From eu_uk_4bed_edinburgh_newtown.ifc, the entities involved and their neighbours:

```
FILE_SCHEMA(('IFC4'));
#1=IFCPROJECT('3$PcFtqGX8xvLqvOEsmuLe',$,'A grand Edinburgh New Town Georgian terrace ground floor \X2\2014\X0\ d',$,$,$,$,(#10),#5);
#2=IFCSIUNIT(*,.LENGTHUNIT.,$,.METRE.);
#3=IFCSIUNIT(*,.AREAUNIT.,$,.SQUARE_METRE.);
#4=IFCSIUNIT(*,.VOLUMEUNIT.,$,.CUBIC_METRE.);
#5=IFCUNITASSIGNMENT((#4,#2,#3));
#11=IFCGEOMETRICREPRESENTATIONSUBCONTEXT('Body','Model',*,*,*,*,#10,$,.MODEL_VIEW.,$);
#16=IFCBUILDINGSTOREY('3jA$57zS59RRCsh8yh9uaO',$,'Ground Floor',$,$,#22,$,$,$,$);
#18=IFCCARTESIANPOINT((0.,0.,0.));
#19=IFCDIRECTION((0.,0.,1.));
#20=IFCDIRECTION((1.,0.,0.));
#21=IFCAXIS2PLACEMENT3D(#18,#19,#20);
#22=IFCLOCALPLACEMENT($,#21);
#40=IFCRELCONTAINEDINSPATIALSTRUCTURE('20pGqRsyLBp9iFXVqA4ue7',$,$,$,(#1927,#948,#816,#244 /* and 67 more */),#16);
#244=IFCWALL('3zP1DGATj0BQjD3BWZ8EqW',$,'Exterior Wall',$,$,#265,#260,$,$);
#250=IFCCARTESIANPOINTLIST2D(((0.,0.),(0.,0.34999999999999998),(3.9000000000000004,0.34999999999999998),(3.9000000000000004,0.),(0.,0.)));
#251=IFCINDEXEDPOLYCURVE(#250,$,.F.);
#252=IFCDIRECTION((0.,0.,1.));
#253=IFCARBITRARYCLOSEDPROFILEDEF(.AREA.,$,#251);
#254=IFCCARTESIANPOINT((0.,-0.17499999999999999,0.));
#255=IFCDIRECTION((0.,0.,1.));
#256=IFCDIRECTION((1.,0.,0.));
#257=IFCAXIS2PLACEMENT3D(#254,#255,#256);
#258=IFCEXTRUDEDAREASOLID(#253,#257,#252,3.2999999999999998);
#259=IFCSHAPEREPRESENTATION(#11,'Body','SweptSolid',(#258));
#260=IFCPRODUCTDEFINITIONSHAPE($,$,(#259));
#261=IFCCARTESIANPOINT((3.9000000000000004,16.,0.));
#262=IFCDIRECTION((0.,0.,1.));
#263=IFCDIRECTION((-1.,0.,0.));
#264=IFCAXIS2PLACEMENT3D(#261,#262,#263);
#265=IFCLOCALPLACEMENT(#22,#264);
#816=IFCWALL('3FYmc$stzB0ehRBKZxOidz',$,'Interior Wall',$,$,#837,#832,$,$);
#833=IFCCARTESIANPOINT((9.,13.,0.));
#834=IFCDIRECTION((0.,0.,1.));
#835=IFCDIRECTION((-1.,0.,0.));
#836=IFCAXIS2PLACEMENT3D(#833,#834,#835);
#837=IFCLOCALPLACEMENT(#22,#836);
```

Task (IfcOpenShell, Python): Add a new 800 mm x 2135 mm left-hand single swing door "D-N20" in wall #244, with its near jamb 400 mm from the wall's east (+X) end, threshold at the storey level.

```python
import numpy as np
import ifcopenshell
import ifcopenshell.api.feature
import ifcopenshell.api.geometry
import ifcopenshell.api.root
import ifcopenshell.api.spatial
import ifcopenshell.geom
import ifcopenshell.util.element
import ifcopenshell.util.placement
import ifcopenshell.util.representation
import ifcopenshell.util.shape
import ifcopenshell.util.unit

model = ifcopenshell.open("eu_uk_4bed_edinburgh_newtown.ifc")
unit_scale = ifcopenshell.util.unit.calculate_unit_scale(model)
settings = ifcopenshell.geom.settings()


def volume(element):
    """Net volume in cubic metres, openings subtracted."""
    shape = ifcopenshell.geom.create_shape(settings, element)
    return ifcopenshell.util.shape.get_volume(shape.geometry)


wall = model.by_guid("3zP1DGATj0BQjD3BWZ8EqW")
storey = ifcopenshell.util.element.get_container(wall, ifc_class="IfcBuildingStorey")
context = ifcopenshell.util.representation.get_context(model, "Model", "Body", "MODEL_VIEW")
before = volume(wall)

width, height, from_end, sill = 0.8, 2.135, 0.4, 0.0  # metres

# The wall runs along its own X axis, and the end named is its -X end.
wall_shape = ifcopenshell.geom.create_shape(settings, wall)
x, y, z = ifcopenshell.util.shape.get_vertices(wall_shape.geometry).T
start = x.min() + from_end
face, thickness = float(y.min()), float(y.max() - y.min())
wall_matrix = ifcopenshell.util.placement.get_local_placement(wall.ObjectPlacement)
level = ifcopenshell.util.placement.get_local_placement(storey.ObjectPlacement)[2, 3]


def in_wall(x, y):
    """Placement at x, y metres in the wall's axes, at sill height."""
    matrix = wall_matrix.copy()
    matrix[:, 3] = wall_matrix @ np.array([x / unit_scale, y / unit_scale, 0.0, 1.0])
    matrix[2, 3] = level + sill / unit_scale
    return matrix


# Opening: a box that overshoots both wall faces by 50 mm.
opening = ifcopenshell.api.root.create_entity(model, ifc_class="IfcOpeningElement", predefined_type="OPENING")
box = ifcopenshell.api.geometry.add_wall_representation(
    model, context=context, length=width, height=height, thickness=thickness + 0.1
)
ifcopenshell.api.geometry.assign_representation(model, product=opening, representation=box)
ifcopenshell.api.geometry.edit_object_placement(model, product=opening, matrix=in_wall(start, face - 0.05), is_si=False)
ifcopenshell.api.feature.add_feature(model, feature=opening, element=wall)

door = ifcopenshell.api.root.create_entity(model, ifc_class="IfcDoor", name="D-N20", predefined_type="DOOR")
door.OverallWidth, door.OverallHeight = width / unit_scale, height / unit_scale
door.OperationType = "SINGLE_SWING_LEFT"
body = ifcopenshell.api.geometry.add_door_representation(
    model,
    context=context,
    overall_width=door.OverallWidth,
    overall_height=door.OverallHeight,
    operation_type="SINGLE_SWING_LEFT",
    lining_properties={"LiningDepth": thickness / unit_scale, "ThresholdDepth": thickness / unit_scale},
)
ifcopenshell.api.geometry.assign_representation(model, product=door, representation=body)
ifcopenshell.api.spatial.assign_container(model, products=[door], relating_structure=storey)
ifcopenshell.api.feature.add_filling(model, opening=opening, element=door)

# The lining spans the wall, so the door starts at the wall face.
ifcopenshell.api.geometry.edit_object_placement(model, product=door, matrix=in_wall(start, face), is_si=False)

after = volume(wall)

print(f"wall volume {before:.3f} -> {after:.3f} m3")

model.write("eu_uk_4bed_edinburgh_newtown_rev.ifc")
```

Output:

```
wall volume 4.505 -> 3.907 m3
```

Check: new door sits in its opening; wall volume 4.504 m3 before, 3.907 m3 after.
